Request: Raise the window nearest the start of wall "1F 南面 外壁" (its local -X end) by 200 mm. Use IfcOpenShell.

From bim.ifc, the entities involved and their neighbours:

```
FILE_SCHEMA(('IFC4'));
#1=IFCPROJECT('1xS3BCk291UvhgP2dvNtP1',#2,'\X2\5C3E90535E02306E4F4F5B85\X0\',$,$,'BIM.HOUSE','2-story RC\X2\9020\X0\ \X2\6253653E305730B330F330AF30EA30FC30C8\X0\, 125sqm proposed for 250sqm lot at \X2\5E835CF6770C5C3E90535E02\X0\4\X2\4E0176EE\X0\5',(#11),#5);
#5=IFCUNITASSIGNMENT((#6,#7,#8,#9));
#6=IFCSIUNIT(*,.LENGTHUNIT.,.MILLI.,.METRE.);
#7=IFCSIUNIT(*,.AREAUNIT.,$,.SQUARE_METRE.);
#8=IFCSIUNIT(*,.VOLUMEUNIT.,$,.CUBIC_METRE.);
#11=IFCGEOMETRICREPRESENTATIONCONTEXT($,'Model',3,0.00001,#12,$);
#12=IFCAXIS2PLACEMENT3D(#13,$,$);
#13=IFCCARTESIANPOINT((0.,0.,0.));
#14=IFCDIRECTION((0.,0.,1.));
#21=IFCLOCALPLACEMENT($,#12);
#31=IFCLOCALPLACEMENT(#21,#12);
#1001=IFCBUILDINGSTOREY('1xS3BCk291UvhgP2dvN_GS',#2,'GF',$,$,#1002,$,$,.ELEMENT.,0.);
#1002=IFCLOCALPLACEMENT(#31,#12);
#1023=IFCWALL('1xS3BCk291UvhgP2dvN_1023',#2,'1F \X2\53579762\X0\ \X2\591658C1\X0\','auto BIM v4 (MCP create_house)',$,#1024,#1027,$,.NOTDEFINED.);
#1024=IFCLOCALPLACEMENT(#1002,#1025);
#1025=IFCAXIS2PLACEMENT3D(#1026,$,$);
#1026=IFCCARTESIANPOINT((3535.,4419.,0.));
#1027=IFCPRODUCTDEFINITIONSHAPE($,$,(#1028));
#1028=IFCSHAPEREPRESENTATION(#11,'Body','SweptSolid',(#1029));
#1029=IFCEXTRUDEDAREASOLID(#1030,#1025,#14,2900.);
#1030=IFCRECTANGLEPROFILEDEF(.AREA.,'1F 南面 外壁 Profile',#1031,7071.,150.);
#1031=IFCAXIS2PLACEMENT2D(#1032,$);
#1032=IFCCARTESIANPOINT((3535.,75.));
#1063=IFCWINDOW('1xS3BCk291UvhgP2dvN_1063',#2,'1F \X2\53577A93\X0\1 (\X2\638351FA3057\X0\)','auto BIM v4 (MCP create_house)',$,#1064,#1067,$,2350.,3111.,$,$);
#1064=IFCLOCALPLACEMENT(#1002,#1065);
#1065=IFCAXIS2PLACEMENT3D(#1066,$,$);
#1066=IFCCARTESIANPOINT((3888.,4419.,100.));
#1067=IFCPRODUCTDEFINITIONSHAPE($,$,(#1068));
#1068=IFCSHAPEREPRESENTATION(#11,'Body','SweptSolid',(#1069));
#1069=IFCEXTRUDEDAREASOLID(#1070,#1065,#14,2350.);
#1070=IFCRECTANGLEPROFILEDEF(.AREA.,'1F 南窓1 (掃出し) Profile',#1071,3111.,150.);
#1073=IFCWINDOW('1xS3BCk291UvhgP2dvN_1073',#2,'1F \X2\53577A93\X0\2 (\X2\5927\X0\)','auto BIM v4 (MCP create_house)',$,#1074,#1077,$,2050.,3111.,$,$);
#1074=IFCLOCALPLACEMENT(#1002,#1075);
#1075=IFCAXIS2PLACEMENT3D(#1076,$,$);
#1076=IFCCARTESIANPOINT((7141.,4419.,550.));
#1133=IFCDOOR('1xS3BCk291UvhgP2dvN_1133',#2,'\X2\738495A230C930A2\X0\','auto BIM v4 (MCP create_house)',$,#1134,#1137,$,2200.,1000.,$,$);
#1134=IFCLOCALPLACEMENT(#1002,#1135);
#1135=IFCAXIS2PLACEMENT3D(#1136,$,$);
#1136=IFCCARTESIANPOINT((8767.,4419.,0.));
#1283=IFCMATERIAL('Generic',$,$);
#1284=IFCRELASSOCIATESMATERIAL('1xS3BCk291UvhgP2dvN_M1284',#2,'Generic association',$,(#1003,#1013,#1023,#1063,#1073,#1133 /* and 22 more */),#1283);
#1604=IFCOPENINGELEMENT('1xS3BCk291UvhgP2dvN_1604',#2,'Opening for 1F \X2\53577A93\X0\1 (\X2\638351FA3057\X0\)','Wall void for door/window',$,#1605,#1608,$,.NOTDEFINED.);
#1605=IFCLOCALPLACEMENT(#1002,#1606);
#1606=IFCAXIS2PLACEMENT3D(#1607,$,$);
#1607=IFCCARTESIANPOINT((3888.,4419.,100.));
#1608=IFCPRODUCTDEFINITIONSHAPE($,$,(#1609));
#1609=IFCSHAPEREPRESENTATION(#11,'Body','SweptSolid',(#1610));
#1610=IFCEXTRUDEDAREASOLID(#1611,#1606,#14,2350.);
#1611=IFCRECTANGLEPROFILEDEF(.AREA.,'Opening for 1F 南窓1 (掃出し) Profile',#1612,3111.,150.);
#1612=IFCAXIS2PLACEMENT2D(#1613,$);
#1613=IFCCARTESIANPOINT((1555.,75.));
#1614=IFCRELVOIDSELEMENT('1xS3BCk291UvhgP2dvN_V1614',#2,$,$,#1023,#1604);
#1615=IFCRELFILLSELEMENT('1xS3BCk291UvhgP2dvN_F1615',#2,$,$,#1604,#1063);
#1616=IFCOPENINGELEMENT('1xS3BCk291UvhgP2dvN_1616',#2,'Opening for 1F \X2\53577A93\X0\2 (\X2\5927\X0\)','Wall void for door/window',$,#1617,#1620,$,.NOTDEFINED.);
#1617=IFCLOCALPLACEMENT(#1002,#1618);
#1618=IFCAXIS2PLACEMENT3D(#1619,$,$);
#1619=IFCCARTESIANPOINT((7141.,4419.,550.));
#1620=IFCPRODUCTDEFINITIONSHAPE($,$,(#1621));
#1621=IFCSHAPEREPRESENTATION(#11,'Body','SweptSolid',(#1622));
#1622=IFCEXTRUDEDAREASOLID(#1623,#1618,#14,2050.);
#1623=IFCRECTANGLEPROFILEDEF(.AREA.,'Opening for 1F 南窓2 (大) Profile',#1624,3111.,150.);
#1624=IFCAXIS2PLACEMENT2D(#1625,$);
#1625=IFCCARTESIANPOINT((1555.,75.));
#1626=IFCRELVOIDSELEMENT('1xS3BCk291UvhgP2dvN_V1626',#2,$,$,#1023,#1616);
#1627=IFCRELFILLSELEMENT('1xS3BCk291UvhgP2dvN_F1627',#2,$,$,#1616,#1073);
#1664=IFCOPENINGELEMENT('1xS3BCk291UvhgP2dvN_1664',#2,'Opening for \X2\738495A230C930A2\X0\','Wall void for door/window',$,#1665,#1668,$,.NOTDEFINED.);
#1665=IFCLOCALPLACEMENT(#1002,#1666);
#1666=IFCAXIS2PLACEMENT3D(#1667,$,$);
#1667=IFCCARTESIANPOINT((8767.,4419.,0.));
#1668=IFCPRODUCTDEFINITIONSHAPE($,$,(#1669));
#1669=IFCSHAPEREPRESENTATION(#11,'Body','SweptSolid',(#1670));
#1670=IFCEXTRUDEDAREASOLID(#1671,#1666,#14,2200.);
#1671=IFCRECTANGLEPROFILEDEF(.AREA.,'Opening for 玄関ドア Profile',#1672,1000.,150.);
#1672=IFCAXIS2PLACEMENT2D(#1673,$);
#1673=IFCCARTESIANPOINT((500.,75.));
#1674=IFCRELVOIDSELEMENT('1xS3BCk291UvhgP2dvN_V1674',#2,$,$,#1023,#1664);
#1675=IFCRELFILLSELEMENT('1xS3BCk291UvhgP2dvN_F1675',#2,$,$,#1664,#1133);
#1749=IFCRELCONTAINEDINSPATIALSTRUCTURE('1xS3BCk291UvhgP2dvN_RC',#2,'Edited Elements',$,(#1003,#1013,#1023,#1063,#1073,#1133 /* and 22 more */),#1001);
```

```python
import numpy as np
import ifcopenshell
import ifcopenshell.api.geometry
import ifcopenshell.util.placement
import ifcopenshell.util.unit

model = ifcopenshell.open("bim.ifc")
unit_scale = ifcopenshell.util.unit.calculate_unit_scale(model)

window = model.by_guid("1xS3BCk291UvhgP2dvN_1063")
opening = window.FillsVoids[0].RelatingOpeningElement
dz = 0.2 / unit_scale

shift = np.array([0.0, 0.0, dz])
# The window is not placed relative to its opening, so move both.
for product in (opening, window):
    matrix = ifcopenshell.util.placement.get_local_placement(product.ObjectPlacement)
    matrix[:3, 3] += shift
    ifcopenshell.api.geometry.edit_object_placement(model, product=product, matrix=matrix, is_si=False)

print(f"moved by {dz * unit_scale:+.3f} m")

model.write("bim-out.ifc")
```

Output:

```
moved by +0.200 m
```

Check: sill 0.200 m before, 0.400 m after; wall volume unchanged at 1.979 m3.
